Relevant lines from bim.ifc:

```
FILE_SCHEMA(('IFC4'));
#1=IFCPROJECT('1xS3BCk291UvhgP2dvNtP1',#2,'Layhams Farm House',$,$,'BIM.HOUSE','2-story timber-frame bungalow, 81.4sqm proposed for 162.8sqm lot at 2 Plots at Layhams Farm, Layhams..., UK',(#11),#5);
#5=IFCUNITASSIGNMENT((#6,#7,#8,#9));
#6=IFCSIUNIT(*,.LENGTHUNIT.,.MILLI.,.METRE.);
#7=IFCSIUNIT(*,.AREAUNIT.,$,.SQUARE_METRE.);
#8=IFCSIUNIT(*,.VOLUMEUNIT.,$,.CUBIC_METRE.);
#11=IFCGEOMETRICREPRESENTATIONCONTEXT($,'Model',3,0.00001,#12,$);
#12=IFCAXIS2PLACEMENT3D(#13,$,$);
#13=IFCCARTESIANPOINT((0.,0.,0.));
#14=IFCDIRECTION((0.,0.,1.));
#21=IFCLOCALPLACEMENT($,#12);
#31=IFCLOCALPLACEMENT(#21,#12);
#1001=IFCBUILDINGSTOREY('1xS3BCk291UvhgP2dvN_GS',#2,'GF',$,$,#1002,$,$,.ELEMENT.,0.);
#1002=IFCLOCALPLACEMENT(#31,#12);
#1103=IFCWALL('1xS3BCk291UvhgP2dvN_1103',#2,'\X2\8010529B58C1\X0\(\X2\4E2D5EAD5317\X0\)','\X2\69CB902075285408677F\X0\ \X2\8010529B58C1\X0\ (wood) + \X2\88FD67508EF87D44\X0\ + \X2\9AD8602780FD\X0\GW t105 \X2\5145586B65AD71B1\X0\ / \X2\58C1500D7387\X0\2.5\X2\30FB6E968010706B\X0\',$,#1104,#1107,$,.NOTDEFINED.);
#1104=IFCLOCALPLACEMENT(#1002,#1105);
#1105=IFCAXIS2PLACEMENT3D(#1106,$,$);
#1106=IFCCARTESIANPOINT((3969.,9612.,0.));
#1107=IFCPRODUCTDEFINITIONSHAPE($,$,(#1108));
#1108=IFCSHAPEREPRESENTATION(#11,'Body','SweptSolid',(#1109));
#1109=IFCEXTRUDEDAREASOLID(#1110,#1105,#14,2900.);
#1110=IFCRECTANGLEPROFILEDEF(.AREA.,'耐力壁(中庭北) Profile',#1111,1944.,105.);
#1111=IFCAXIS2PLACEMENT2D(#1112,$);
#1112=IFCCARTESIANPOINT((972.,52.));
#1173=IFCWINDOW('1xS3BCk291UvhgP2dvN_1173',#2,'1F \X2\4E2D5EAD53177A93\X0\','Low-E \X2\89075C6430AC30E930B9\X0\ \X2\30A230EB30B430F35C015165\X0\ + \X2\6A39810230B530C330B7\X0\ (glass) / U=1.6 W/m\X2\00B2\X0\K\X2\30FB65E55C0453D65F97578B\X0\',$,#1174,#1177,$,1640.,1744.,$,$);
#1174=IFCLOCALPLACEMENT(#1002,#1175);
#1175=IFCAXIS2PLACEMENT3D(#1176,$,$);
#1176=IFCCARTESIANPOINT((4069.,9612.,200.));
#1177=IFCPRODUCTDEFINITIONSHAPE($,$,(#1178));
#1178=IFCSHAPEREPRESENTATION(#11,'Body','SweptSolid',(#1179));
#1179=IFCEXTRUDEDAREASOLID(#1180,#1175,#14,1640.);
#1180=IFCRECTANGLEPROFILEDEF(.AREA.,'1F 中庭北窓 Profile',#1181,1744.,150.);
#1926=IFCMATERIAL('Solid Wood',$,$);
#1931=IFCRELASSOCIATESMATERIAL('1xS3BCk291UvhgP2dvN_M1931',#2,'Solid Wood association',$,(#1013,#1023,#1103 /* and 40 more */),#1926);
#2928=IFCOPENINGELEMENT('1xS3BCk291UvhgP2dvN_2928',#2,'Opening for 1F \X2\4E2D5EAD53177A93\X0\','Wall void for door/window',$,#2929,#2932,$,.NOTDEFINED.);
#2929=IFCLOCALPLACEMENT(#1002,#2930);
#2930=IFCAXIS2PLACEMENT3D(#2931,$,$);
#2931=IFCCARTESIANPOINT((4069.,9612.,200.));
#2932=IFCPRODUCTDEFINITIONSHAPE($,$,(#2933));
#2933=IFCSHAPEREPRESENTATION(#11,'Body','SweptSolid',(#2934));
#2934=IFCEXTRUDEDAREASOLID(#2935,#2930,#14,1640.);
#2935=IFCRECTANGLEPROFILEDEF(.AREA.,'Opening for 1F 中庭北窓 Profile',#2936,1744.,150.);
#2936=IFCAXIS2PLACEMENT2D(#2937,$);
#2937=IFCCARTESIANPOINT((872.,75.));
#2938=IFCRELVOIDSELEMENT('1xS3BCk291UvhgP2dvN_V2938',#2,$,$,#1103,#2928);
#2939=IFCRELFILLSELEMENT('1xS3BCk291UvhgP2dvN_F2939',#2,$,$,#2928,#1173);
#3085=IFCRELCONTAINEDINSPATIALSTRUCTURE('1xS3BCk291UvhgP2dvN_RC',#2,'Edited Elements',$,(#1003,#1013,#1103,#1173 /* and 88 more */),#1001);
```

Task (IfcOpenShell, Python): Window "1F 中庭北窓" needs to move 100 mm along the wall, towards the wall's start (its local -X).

```python
import ifcopenshell
import ifcopenshell.api.geometry
import ifcopenshell.util.placement
import ifcopenshell.util.unit

model = ifcopenshell.open("bim.ifc")
unit_scale = ifcopenshell.util.unit.calculate_unit_scale(model)

window = model.by_guid("1xS3BCk291UvhgP2dvN_1173")
opening = window.FillsVoids[0].RelatingOpeningElement
wall = opening.VoidsElements[0].RelatingBuildingElement

wall_matrix = ifcopenshell.util.placement.get_local_placement(wall.ObjectPlacement)
shift = wall_matrix[:3, 0] * -0.1 / unit_scale
before = ifcopenshell.util.placement.get_local_placement(window.ObjectPlacement)[:3, 3].copy()

# The window is not placed relative to its opening, so move both.
for product in (opening, window):
    matrix = ifcopenshell.util.placement.get_local_placement(product.ObjectPlacement)
    matrix[:3, 3] += shift
    ifcopenshell.api.geometry.edit_object_placement(model, product=product, matrix=matrix, is_si=False)

after = ifcopenshell.util.placement.get_local_placement(window.ObjectPlacement)[:3, 3]
print("window moved by", (after - before).round(3) + 0.0)

model.write("bim_v2.ifc")
```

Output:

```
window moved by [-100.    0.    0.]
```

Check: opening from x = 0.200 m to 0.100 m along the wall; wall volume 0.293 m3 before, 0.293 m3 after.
